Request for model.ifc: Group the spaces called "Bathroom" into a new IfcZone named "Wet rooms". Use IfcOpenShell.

First a look at what the model holds.

```python
import ifcopenshell

model = ifcopenshell.open("model.ifc")
print(model.schema)
seen = {}
for space in model.by_type("IfcSpace"):
    seen[space.LongName] = seen.get(space.LongName, 0) + 1
for name, count in sorted(seen.items(), key=str):
    print(count, "x", name)
print("zones:", [z.Name for z in model.by_type("IfcZone")][:20])
```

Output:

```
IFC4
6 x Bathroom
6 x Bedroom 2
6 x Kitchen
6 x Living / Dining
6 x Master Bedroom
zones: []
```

```python
import ifcopenshell
import ifcopenshell.api.group
import ifcopenshell.api.root

model = ifcopenshell.open("model.ifc")

names = {"Bathroom"}
spaces = [s for s in model.by_type("IfcSpace") if s.LongName in names]

zone = ifcopenshell.api.root.create_entity(model, ifc_class="IfcZone", name="Wet rooms")
ifcopenshell.api.group.assign_group(model, products=spaces, group=zone)
print(len(spaces), "spaces in", zone.Name)

model.write("model_v2.ifc")
```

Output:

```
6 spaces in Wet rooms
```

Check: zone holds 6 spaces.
